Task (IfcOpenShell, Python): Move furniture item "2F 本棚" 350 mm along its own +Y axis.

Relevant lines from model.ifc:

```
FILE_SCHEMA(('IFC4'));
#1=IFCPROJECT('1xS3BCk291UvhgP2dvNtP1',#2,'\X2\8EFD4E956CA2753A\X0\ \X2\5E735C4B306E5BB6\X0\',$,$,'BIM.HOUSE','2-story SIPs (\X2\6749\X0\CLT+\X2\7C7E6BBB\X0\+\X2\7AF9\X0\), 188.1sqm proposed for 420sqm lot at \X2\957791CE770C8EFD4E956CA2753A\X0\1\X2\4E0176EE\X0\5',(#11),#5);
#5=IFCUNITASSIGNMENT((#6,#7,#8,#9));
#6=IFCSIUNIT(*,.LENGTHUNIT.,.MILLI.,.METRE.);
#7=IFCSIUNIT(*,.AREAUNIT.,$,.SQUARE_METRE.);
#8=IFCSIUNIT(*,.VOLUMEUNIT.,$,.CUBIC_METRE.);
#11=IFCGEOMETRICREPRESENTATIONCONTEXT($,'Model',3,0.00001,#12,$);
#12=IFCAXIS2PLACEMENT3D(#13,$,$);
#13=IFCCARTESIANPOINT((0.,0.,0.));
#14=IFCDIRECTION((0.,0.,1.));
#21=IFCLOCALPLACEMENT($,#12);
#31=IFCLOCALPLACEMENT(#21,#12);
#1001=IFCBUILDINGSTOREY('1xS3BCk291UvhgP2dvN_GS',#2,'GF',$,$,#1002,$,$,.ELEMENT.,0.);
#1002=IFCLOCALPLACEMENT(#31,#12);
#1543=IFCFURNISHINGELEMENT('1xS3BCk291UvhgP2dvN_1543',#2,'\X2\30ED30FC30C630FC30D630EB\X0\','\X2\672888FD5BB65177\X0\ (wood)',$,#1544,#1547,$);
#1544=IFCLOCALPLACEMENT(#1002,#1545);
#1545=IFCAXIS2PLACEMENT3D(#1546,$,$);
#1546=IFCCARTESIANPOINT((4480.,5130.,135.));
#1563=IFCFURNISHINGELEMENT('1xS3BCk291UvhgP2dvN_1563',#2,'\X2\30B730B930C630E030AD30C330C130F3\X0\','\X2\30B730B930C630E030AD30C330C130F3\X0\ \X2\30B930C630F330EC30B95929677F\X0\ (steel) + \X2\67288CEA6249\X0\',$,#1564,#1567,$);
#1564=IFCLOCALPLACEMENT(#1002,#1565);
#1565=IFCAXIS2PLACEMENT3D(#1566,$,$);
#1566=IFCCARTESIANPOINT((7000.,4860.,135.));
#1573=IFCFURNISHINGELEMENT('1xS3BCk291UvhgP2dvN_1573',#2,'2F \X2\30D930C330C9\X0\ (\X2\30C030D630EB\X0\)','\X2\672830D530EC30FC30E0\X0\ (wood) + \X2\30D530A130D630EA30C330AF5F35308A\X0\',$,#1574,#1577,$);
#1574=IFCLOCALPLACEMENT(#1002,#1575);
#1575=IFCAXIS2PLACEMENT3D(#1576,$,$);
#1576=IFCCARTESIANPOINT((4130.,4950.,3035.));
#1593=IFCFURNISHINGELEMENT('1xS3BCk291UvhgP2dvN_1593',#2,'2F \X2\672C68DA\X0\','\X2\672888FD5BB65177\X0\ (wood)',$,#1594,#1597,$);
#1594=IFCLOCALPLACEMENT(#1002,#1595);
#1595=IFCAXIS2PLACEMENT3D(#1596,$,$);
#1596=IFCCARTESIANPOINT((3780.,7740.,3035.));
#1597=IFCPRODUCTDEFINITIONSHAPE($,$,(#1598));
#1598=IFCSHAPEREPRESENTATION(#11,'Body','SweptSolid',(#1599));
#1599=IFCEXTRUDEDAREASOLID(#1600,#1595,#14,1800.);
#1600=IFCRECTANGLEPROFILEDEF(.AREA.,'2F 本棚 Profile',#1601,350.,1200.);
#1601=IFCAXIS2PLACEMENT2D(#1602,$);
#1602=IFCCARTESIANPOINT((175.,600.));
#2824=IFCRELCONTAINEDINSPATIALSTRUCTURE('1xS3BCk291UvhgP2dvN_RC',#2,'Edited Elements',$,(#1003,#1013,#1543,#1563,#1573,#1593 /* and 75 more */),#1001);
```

```python
import ifcopenshell
import ifcopenshell.api.geometry
import ifcopenshell.util.placement

model = ifcopenshell.open("model.ifc")

item = model.by_id(1593)
matrix = ifcopenshell.util.placement.get_local_placement(item.ObjectPlacement)
matrix[:3, 3] += matrix[:3, 1] * 350.0
ifcopenshell.api.geometry.edit_object_placement(model, product=item, matrix=matrix, is_si=False)

print(ifcopenshell.util.placement.get_local_placement(item.ObjectPlacement).round(3) + 0.0)

model.write("model_v2.ifc")
```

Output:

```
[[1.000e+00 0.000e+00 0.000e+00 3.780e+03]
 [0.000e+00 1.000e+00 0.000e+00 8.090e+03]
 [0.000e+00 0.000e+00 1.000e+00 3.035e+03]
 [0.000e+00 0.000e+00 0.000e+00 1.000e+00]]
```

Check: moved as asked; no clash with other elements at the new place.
